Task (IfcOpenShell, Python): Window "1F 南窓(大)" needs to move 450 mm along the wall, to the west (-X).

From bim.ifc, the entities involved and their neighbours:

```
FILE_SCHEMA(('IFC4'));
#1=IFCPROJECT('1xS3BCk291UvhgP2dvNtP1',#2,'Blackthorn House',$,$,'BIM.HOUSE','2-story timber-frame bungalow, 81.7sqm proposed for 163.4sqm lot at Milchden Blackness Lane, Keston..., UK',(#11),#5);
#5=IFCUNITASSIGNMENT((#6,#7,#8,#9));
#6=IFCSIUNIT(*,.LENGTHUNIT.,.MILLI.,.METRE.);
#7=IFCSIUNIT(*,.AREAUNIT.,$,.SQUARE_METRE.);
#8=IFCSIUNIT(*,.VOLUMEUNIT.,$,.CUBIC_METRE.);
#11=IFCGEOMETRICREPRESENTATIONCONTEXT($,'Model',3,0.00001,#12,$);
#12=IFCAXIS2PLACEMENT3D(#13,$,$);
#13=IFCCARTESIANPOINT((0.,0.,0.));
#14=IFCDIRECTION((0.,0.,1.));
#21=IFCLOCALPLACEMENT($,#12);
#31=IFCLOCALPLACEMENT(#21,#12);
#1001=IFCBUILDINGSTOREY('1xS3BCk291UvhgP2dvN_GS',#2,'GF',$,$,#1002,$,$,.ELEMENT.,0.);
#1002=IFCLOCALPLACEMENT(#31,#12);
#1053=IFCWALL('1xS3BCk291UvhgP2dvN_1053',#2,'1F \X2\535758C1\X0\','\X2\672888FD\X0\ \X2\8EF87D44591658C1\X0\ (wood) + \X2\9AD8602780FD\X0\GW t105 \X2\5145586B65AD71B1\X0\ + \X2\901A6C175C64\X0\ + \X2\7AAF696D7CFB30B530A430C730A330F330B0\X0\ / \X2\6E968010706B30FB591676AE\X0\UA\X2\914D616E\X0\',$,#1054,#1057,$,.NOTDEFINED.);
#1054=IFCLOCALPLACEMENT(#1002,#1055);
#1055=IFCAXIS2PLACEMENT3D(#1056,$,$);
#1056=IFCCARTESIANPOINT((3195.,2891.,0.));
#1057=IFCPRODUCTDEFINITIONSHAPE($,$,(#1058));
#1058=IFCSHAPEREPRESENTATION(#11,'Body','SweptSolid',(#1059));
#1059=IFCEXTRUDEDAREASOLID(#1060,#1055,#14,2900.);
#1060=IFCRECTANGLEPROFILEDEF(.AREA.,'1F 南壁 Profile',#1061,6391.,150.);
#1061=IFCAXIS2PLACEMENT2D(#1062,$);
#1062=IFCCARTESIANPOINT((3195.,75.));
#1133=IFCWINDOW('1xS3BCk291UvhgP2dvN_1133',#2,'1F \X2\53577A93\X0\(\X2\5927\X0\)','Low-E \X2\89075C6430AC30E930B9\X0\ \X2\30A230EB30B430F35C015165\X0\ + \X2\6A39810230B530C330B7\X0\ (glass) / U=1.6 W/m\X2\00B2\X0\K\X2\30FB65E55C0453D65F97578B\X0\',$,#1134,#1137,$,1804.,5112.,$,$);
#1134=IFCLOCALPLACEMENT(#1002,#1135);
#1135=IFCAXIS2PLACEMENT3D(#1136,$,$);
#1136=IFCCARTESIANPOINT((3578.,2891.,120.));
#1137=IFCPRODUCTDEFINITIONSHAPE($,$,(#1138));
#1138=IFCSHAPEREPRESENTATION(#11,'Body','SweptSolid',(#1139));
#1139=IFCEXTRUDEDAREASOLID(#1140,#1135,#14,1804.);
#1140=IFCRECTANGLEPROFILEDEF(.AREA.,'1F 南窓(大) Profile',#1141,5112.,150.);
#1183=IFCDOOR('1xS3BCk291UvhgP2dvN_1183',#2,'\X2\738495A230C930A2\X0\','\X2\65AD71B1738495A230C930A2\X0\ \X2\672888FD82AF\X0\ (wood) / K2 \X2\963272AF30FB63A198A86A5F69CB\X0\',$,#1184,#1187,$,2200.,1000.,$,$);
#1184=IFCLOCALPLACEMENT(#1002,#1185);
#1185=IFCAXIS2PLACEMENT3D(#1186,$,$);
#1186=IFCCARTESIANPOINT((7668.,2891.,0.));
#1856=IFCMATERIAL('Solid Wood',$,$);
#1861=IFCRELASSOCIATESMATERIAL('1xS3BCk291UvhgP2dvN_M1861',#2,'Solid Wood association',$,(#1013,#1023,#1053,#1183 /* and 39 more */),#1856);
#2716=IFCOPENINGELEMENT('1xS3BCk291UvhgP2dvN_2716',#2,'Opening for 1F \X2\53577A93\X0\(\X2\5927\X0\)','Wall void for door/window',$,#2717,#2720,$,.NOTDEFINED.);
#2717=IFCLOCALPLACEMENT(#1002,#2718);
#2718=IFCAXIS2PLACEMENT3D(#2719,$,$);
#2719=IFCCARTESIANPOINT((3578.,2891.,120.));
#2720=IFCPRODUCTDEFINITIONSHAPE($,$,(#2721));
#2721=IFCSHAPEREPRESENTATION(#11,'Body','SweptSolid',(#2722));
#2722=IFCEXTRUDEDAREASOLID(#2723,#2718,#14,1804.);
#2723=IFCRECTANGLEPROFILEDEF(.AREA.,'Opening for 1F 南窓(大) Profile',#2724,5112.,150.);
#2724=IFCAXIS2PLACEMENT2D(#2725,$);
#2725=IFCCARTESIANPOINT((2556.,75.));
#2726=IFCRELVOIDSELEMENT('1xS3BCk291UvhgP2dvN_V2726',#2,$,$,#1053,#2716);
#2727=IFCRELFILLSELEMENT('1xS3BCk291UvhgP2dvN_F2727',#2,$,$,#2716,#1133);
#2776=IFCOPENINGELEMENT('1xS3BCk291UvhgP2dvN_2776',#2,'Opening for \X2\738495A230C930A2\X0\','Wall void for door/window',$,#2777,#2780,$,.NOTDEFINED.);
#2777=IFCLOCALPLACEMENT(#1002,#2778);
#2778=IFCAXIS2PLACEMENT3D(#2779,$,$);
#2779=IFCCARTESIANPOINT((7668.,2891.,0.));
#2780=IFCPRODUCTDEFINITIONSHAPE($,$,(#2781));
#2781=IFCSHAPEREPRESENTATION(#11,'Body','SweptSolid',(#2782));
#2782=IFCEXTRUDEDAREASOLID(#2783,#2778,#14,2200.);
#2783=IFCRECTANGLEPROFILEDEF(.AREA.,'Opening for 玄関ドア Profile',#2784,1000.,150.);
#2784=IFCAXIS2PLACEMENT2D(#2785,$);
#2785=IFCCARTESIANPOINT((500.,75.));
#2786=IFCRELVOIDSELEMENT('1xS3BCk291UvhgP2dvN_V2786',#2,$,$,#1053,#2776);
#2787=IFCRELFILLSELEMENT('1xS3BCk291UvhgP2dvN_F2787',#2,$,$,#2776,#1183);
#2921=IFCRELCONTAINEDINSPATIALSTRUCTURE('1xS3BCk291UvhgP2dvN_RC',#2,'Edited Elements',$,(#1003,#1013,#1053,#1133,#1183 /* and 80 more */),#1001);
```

```python
import ifcopenshell
import ifcopenshell.api.geometry
import ifcopenshell.util.placement

model = ifcopenshell.open("bim.ifc")

window = model.by_id(1133)
opening = window.FillsVoids[0].RelatingOpeningElement
wall = opening.VoidsElements[0].RelatingBuildingElement

wall_matrix = ifcopenshell.util.placement.get_local_placement(wall.ObjectPlacement)
shift = wall_matrix[:3, 0] * -450.0
before = ifcopenshell.util.placement.get_local_placement(window.ObjectPlacement)[:3, 3].copy()

# The window is not placed relative to its opening, so move both.
for product in (opening, window):
    matrix = ifcopenshell.util.placement.get_local_placement(product.ObjectPlacement)
    matrix[:3, 3] += shift
    ifcopenshell.api.geometry.edit_object_placement(model, product=product, matrix=matrix, is_si=False)

after = ifcopenshell.util.placement.get_local_placement(window.ObjectPlacement)[:3, 3]
print("window moved by", (after - before).round(3) + 0.0)

model.write("bim_edited.ifc")
```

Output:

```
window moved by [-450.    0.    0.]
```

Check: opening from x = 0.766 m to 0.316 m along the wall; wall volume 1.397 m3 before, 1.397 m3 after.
